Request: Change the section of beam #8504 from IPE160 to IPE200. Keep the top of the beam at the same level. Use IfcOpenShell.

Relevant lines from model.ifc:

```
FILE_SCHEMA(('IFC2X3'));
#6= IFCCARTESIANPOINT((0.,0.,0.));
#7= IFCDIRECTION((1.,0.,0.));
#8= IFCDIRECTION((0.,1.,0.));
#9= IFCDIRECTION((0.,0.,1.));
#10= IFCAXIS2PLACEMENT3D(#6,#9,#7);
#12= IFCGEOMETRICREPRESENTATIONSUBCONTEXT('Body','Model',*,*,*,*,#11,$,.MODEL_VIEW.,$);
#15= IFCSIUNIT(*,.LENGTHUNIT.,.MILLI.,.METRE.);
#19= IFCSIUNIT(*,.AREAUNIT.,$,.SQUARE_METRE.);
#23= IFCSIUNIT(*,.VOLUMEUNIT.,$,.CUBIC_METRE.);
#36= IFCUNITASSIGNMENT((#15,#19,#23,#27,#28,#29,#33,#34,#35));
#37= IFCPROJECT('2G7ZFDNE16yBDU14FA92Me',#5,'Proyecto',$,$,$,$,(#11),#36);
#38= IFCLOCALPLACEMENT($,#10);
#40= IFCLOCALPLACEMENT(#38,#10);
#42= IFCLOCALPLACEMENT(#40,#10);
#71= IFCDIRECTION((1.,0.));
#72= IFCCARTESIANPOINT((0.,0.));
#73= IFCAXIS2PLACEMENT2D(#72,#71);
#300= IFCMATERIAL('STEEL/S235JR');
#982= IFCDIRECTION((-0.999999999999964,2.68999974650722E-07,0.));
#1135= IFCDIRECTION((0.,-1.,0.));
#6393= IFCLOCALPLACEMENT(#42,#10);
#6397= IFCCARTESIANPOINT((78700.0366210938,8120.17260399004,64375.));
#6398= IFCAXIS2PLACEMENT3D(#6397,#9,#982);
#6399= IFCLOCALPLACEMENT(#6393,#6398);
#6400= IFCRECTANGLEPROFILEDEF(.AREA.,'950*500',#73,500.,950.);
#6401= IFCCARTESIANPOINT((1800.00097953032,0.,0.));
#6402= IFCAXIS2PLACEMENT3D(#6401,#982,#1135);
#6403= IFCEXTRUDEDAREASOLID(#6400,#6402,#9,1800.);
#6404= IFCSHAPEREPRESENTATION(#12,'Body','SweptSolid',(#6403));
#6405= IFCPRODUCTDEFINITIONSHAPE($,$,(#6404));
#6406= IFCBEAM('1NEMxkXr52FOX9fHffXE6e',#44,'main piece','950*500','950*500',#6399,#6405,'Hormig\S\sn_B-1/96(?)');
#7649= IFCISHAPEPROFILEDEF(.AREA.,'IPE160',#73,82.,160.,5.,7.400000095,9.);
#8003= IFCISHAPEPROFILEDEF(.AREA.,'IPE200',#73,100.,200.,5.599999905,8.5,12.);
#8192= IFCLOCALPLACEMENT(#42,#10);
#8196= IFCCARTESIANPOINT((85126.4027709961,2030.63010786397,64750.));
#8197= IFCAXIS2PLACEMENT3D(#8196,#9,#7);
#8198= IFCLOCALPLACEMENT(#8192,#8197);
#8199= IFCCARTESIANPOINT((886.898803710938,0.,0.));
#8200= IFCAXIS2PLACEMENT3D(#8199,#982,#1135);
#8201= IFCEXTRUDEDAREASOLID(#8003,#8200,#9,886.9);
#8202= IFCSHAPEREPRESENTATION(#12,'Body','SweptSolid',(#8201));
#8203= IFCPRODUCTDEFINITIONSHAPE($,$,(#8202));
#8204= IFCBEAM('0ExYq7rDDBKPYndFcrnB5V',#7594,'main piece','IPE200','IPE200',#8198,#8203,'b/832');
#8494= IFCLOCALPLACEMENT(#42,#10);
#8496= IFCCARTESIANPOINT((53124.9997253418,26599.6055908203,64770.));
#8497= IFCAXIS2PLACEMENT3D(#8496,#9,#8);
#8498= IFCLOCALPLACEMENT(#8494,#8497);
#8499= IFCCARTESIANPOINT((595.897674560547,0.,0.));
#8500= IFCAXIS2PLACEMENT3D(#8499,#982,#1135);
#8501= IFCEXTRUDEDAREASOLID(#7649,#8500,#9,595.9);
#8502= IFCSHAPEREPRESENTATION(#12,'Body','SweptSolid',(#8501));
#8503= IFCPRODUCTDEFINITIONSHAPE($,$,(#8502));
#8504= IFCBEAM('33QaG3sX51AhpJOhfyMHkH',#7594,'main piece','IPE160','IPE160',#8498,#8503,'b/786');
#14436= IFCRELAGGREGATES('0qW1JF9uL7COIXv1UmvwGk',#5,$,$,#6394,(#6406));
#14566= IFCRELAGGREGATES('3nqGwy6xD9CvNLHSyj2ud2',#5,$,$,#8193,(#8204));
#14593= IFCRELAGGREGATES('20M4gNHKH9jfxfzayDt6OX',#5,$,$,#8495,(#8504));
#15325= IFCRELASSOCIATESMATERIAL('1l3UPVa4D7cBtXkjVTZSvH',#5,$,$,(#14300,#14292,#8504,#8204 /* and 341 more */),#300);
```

```python
import ifcopenshell
import ifcopenshell.util.element
import ifcopenshell.util.representation

model = ifcopenshell.open("model.ifc")

member = model.by_guid("33QaG3sX51AhpJOhfyMHkH")
source = next(p for p in model.by_type("IfcIShapeProfileDef") if p.ProfileName == "IPE200")

body = ifcopenshell.util.representation.get_representation(member, "Model", "Body")
solid = body.Items[0]
old_profile = solid.SweptArea

# Copy the section's sizes but keep this member's own profile position.
profile = ifcopenshell.util.element.copy(model, source)
# Profiles are centred, so shift by half the change in depth to hold the top.
shift = (old_profile.OverallDepth - profile.OverallDepth) / 2
x, y = old_profile.Position.Location.Coordinates
up = (0.0, 1.0)  # upwards, in the solid's own plane
location = model.createIfcCartesianPoint((x + up[0] * shift, y + up[1] * shift))
profile.Position = model.createIfcAxis2Placement2D(location, old_profile.Position.RefDirection)
solid.SweptArea = profile
if not model.get_total_inverses(old_profile):
    ifcopenshell.util.element.remove_deep2(model, old_profile)
member.Description = member.Description.replace("IPE160", "IPE200")
member.ObjectType = member.ObjectType.replace("IPE160", "IPE200")

print(solid.SweptArea)

model.write("model_edited.ifc")
```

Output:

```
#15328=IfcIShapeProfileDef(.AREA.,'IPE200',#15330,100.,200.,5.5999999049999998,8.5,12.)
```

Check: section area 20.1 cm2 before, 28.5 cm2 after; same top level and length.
